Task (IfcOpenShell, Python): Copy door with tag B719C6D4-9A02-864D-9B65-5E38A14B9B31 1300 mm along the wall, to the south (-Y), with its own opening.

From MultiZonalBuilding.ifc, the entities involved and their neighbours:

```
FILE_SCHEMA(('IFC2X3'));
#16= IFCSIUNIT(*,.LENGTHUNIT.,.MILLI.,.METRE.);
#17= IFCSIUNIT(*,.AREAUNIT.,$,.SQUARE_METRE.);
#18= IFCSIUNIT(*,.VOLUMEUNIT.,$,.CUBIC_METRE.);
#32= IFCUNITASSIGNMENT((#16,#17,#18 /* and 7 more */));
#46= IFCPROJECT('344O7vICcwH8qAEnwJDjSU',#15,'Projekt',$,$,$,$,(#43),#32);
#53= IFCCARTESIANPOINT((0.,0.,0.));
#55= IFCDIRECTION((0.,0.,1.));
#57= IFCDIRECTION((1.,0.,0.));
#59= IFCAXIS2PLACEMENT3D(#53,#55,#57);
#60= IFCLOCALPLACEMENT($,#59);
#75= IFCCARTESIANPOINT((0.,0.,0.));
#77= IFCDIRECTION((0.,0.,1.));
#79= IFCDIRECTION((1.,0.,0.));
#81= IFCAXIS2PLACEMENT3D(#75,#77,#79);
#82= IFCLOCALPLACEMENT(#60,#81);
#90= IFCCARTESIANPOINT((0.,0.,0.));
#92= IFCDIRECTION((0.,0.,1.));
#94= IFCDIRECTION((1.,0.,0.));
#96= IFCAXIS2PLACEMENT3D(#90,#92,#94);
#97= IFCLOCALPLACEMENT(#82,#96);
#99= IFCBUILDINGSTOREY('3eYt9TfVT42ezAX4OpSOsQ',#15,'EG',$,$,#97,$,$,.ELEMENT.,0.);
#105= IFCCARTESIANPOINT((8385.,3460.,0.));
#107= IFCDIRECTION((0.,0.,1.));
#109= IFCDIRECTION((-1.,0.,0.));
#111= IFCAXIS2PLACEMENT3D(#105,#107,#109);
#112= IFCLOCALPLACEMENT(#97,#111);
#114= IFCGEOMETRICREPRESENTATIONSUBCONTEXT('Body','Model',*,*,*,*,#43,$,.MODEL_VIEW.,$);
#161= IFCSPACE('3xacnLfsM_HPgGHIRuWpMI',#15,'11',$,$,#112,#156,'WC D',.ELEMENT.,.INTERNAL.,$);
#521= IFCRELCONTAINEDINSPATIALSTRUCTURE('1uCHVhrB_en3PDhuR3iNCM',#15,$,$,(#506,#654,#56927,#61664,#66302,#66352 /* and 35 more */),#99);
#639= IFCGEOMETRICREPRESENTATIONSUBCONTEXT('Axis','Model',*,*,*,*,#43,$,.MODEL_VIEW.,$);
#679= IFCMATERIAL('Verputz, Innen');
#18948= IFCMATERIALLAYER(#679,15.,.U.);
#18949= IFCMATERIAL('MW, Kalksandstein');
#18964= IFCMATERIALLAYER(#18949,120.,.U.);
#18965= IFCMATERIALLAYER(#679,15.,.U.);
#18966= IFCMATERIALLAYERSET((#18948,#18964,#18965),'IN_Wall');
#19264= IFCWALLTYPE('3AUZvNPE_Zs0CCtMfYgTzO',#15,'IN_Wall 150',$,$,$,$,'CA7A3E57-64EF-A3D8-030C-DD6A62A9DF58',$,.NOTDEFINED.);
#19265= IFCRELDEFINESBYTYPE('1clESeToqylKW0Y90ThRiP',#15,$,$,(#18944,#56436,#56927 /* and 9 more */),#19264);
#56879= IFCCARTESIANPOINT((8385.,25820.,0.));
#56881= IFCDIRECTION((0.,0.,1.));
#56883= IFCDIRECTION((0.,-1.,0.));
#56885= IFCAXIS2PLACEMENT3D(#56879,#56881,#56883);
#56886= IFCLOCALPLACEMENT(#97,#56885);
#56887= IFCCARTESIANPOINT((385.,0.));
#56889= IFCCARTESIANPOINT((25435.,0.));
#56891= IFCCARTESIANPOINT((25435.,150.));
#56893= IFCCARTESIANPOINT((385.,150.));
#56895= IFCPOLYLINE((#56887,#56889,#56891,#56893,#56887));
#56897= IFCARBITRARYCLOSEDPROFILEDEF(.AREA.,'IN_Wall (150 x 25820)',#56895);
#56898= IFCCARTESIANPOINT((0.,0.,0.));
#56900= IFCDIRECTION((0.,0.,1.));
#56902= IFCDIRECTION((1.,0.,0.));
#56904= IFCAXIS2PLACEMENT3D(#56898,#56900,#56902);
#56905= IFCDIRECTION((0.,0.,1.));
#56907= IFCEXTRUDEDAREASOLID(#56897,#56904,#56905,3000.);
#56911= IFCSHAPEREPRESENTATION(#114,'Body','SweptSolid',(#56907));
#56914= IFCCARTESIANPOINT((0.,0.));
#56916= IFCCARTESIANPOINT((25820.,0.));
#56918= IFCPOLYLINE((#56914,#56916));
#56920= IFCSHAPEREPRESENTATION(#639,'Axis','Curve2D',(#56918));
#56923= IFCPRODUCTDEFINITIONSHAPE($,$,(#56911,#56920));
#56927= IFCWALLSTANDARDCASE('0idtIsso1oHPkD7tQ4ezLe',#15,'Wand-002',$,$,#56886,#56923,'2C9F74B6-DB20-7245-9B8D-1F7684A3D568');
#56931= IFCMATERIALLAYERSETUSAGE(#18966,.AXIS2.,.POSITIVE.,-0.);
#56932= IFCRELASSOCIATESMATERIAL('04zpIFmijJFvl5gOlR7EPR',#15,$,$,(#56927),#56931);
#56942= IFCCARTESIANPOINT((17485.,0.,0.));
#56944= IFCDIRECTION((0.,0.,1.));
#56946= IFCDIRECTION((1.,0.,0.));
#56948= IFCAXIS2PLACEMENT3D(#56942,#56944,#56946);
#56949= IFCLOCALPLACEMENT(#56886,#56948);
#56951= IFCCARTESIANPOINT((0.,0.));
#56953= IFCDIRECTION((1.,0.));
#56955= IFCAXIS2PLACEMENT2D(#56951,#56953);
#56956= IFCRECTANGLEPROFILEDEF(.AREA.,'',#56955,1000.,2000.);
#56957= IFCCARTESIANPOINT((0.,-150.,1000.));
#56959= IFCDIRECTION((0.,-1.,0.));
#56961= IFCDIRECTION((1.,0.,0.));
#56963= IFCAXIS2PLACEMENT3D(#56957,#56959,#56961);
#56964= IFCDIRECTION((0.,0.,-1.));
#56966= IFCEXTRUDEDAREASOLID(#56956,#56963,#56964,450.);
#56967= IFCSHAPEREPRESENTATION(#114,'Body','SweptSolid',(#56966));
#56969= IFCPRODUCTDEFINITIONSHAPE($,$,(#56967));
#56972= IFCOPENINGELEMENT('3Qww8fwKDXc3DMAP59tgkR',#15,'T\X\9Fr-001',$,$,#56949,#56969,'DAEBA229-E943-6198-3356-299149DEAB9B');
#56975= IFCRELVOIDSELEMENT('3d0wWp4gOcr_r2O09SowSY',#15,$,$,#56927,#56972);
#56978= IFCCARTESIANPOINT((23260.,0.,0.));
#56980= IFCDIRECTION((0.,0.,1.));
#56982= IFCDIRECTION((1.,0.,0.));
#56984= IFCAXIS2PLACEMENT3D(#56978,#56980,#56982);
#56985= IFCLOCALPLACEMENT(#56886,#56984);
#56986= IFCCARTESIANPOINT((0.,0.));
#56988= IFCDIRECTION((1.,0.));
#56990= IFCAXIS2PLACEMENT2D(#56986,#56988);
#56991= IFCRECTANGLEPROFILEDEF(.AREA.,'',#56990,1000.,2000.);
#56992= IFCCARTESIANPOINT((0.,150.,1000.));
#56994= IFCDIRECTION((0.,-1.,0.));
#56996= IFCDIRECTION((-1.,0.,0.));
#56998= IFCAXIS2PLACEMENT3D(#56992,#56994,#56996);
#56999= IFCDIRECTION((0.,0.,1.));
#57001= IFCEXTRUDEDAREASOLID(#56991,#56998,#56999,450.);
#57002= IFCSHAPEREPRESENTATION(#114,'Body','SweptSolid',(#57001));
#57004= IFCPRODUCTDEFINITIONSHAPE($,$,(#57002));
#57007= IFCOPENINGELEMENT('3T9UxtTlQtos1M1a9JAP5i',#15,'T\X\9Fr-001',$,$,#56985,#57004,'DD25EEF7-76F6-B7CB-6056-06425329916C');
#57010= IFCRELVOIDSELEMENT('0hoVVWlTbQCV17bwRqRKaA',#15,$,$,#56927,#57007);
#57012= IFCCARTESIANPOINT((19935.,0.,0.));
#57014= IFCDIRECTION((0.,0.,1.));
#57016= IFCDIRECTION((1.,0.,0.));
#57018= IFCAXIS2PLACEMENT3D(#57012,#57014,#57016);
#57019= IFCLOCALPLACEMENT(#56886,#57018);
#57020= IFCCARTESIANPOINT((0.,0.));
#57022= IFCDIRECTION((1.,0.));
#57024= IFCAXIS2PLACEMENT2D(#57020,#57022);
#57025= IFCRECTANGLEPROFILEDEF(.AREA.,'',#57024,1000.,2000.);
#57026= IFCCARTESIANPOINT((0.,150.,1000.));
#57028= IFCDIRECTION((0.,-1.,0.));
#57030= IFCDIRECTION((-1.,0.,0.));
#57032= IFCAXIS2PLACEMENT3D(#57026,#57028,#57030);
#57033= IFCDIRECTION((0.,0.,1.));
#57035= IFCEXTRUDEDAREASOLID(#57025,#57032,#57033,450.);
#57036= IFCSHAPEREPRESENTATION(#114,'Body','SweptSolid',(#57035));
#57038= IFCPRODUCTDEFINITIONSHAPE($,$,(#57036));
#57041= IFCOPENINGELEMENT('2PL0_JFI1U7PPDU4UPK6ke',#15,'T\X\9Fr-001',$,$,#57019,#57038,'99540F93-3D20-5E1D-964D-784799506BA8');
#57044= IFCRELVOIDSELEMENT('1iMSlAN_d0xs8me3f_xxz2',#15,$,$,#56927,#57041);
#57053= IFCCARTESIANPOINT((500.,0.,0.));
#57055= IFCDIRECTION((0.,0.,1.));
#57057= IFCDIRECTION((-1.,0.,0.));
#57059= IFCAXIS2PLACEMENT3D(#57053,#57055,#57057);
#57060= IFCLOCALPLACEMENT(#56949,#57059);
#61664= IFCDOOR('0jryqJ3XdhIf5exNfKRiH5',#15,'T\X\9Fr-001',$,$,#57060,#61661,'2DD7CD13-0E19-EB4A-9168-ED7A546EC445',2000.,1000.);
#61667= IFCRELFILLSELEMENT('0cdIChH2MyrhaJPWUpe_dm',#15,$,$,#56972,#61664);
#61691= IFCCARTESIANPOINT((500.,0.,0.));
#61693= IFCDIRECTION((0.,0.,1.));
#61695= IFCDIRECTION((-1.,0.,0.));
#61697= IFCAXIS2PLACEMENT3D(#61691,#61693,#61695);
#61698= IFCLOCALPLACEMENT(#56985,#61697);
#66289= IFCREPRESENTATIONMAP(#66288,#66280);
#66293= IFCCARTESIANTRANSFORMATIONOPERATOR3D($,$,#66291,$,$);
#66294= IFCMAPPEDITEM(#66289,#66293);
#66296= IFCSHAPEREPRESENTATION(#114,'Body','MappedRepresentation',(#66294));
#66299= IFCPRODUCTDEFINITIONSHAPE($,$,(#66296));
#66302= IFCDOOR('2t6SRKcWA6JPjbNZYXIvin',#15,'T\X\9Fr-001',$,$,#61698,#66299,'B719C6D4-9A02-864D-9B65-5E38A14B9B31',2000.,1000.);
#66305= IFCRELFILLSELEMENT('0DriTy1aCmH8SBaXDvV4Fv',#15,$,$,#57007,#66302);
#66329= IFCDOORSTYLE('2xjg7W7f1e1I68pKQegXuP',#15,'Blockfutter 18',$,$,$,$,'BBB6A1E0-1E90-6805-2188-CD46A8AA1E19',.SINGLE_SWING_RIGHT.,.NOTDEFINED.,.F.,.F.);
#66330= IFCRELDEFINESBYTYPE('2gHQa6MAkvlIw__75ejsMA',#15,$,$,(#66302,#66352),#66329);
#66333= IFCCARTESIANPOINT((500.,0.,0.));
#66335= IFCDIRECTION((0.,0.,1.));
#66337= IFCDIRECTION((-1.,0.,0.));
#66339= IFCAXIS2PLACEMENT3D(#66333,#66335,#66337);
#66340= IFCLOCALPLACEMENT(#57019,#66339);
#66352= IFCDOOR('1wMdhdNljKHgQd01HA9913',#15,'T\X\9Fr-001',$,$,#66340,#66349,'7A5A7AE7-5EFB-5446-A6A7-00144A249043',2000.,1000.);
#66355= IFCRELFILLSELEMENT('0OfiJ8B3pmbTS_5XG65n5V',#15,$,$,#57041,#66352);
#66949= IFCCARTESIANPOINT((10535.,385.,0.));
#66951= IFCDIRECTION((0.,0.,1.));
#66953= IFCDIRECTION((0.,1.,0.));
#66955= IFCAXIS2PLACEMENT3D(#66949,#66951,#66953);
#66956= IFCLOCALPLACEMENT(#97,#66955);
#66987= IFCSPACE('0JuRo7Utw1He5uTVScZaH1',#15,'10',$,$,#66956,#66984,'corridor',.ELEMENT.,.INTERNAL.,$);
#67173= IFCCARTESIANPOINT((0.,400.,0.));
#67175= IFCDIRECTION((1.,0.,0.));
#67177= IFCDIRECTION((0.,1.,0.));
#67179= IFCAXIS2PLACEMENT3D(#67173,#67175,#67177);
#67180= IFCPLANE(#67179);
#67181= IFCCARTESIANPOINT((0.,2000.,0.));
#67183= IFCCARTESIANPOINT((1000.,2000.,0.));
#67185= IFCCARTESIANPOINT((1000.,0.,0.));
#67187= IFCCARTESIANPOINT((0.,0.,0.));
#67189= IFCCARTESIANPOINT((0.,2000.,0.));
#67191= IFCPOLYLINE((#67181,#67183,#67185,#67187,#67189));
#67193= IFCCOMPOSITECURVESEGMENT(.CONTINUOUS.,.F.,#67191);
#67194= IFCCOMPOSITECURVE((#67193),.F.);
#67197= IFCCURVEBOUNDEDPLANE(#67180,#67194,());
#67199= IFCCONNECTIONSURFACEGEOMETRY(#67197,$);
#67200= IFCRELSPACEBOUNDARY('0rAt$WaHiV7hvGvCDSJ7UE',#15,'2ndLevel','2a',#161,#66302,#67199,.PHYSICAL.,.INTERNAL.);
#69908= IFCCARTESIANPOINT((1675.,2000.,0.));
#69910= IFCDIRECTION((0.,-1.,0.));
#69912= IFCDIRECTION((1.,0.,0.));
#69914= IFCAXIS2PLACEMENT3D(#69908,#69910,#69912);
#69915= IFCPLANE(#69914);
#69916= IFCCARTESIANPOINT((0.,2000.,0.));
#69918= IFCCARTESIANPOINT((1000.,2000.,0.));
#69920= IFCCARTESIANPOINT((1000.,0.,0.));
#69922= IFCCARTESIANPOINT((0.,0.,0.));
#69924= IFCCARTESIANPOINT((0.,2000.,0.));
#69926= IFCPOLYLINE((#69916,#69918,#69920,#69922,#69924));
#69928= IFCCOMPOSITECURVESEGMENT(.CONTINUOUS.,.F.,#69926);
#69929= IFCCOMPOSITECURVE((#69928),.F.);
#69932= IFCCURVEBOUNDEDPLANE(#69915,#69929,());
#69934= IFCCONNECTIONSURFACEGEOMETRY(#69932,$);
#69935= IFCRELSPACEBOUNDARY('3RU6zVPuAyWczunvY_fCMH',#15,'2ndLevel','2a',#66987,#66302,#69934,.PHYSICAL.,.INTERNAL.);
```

```python
import numpy as np
import ifcopenshell
import ifcopenshell.api.feature
import ifcopenshell.api.geometry
import ifcopenshell.api.root
import ifcopenshell.geom
import ifcopenshell.util.element
import ifcopenshell.util.placement
import ifcopenshell.util.shape
import ifcopenshell.util.unit

model = ifcopenshell.open("MultiZonalBuilding.ifc")
unit_scale = ifcopenshell.util.unit.calculate_unit_scale(model)
settings = ifcopenshell.geom.settings()


def volume(element):
    """Net volume in cubic metres, openings subtracted."""
    shape = ifcopenshell.geom.create_shape(settings, element)
    return ifcopenshell.util.shape.get_volume(shape.geometry)


def reuse_history(source, copy):
    """copy_class also copies each property set's owner history, people and application; keep the originals."""
    for rel in copy.IsDefinedBy:
        if rel.is_a("IfcRelDefinesByProperties") and (history := rel.RelatingPropertyDefinition.OwnerHistory):
            rel.RelatingPropertyDefinition.OwnerHistory = source.OwnerHistory
            ifcopenshell.util.element.remove_deep2(model, history)


door = model.by_guid("2t6SRKcWA6JPjbNZYXIvin")
opening = door.FillsVoids[0].RelatingOpeningElement
wall = opening.VoidsElements[0].RelatingBuildingElement
before = volume(wall)
shift = ifcopenshell.util.placement.get_local_placement(wall.ObjectPlacement)[:3, 0] * 1.3 / unit_scale

# copy_class copies the void relationship, type, container and properties, but no geometry.
new_opening = ifcopenshell.api.root.copy_class(model, product=opening)
new_opening.Representation = ifcopenshell.util.element.copy_deep(
    model, opening.Representation, exclude=["IfcGeometricRepresentationContext", "IfcRepresentationMap"]
)
new_opening.Tag = None
new_door = ifcopenshell.api.root.copy_class(model, product=door)
new_door.Representation = ifcopenshell.util.element.copy_deep(
    model, door.Representation, exclude=["IfcGeometricRepresentationContext", "IfcRepresentationMap"]
)
new_door.Tag = None
reuse_history(door, new_door)
fills = ifcopenshell.api.feature.add_filling(model, opening=new_opening, element=new_door)
fills.OwnerHistory = new_door.OwnerHistory  # required in IFC2X3

for old, new in ((opening, new_opening), (door, new_door)):
    matrix = ifcopenshell.util.placement.get_local_placement(old.ObjectPlacement)
    matrix[:3, 3] += shift
    ifcopenshell.api.geometry.edit_object_placement(model, product=new, matrix=matrix, is_si=False)

# The copied space boundaries still share their surfaces with the original.
for rel in new_door.ProvidesBoundaries:
    if rel.ConnectionGeometry:
        rel.ConnectionGeometry = ifcopenshell.util.element.copy_deep(model, rel.ConnectionGeometry)

# Space boundary surfaces are stored in each space's coordinates; move them too.
for rel in new_door.ProvidesBoundaries:
    if not rel.ConnectionGeometry:
        continue
    surface = rel.ConnectionGeometry.SurfaceOnRelatingElement.BasisSurface
    space_matrix = ifcopenshell.util.placement.get_local_placement(rel.RelatingSpace.ObjectPlacement)
    point = np.array(surface.Position.Location.Coordinates) + space_matrix[:3, :3].T @ shift
    surface.Position = model.createIfcAxis2Placement3D(
        model.createIfcCartesianPoint(point.tolist()), surface.Position.Axis, surface.Position.RefDirection
    )

after = volume(wall)

print(f"wall volume {before:.3f} -> {after:.3f} m3")

model.write("MultiZonalBuilding_updated.ifc")
```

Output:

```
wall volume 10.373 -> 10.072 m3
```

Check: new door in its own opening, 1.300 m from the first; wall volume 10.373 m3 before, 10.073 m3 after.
